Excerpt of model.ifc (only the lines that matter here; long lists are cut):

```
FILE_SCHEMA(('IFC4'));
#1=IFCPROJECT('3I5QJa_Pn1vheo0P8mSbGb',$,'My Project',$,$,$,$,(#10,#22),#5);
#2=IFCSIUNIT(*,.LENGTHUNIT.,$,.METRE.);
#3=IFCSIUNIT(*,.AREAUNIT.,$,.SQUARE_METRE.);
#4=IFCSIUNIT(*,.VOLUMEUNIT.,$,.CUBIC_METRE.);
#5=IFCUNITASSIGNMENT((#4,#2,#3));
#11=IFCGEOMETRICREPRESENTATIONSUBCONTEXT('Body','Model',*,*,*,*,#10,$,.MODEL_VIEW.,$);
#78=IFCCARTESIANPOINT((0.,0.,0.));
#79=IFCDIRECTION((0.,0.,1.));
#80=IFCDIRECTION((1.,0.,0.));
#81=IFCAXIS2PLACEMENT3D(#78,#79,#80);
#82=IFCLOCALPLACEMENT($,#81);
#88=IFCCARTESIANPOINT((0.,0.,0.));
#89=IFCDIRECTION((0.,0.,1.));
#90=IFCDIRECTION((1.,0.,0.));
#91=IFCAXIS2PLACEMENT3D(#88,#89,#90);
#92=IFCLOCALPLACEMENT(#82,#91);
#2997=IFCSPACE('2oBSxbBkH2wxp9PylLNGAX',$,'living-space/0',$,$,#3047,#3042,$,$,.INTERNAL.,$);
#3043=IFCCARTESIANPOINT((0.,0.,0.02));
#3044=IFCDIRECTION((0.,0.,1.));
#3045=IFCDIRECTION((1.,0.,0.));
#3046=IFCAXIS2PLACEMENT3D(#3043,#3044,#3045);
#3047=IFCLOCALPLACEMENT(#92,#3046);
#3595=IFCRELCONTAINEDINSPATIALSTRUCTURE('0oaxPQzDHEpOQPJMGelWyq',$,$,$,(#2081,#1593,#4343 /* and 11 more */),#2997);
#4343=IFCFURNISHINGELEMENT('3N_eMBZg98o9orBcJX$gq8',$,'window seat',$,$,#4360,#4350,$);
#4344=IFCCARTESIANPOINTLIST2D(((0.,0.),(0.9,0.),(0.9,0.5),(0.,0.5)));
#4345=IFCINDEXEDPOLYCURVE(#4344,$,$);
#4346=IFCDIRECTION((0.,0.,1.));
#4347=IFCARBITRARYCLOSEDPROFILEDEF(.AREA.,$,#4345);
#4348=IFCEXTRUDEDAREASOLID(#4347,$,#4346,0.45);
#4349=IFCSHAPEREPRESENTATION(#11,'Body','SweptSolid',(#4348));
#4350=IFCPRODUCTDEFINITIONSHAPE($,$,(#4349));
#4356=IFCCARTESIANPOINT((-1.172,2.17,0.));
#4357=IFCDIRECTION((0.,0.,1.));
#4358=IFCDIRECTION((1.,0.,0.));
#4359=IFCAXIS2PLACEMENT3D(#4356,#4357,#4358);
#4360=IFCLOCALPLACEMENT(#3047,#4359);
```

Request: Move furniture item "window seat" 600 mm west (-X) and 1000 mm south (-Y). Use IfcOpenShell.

```python
import ifcopenshell
import ifcopenshell.api.geometry
import ifcopenshell.util.placement

model = ifcopenshell.open("model.ifc")

item = model.by_guid("3N_eMBZg98o9orBcJX$gq8")
matrix = ifcopenshell.util.placement.get_local_placement(item.ObjectPlacement)
matrix[0, 3] -= 0.6
matrix[1, 3] -= 1.0
ifcopenshell.api.geometry.edit_object_placement(model, product=item, matrix=matrix, is_si=False)

print(ifcopenshell.util.placement.get_local_placement(item.ObjectPlacement).round(3) + 0.0)

model.write("model_edited.ifc")
```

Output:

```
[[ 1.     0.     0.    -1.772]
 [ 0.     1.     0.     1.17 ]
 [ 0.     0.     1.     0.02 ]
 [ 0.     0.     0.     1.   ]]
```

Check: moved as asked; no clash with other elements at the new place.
